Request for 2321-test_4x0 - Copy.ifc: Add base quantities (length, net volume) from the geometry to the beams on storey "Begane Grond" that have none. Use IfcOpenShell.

First a look at what the model holds.

```python
import ifcopenshell
import ifcopenshell.util.element
import ifcopenshell.util.unit

model = ifcopenshell.open("2321-test_4x0 - Copy.ifc")
print(model.schema)
for unit_type in ("LENGTHUNIT", "AREAUNIT", "VOLUMEUNIT"):
    print(unit_type, ifcopenshell.util.unit.calculate_unit_scale(model, unit_type))
storey = next(s for s in model.by_type("IfcBuildingStorey") if s.Name == "Begane Grond")
beams = [e for e in ifcopenshell.util.element.get_decomposition(storey) if e.is_a("IfcBeam")]
for e in sorted(beams, key=lambda e: e.id()):
    print(e.id(), e.is_a(), e.Name, list(ifcopenshell.util.element.get_psets(e, qtos_only=True)), sep=" | ")
```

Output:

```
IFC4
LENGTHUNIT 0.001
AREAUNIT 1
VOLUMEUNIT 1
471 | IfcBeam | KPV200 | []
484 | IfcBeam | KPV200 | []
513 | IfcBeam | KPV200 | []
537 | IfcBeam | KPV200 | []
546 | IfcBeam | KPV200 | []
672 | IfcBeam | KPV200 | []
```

```python
import ifcopenshell
import ifcopenshell.api.pset
import ifcopenshell.geom
import ifcopenshell.util.element
import ifcopenshell.util.shape
import ifcopenshell.util.unit

model = ifcopenshell.open("2321-test_4x0 - Copy.ifc")
unit_scale = ifcopenshell.util.unit.calculate_unit_scale(model)
volume_scale = ifcopenshell.util.unit.calculate_unit_scale(model, "VOLUMEUNIT")
settings = ifcopenshell.geom.settings()

storey = next(s for s in model.by_type("IfcBuildingStorey") if s.Name == "Begane Grond")
beams = [e for e in ifcopenshell.util.element.get_decomposition(storey) if e.is_a("IfcBeam")]

for e in sorted(beams, key=lambda e: e.id()):
    if ifcopenshell.util.element.get_psets(e, qtos_only=True, should_inherit=False):
        continue
    # Geometry comes back in metres, in the element's own axes.
    shape = ifcopenshell.geom.create_shape(settings, e)
    values = {
        "Length": ifcopenshell.util.shape.get_max_xyz(shape.geometry) / unit_scale,
        "NetVolume": ifcopenshell.util.shape.get_volume(shape.geometry) / volume_scale,
    }
    qto = ifcopenshell.api.pset.add_qto(model, product=e, name="Qto_BeamBaseQuantities")
    ifcopenshell.api.pset.edit_qto(model, qto=qto, properties=values)
    print(e.id(), {k: round(v, 3) for k, v in values.items()})

model.write("2321-test_4x0 - Copy_v2.ifc")
```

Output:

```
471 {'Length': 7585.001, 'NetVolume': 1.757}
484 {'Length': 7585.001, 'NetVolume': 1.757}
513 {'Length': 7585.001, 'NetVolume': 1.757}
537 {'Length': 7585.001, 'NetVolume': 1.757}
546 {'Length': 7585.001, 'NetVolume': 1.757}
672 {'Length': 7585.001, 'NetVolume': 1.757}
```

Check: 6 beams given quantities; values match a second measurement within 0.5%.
